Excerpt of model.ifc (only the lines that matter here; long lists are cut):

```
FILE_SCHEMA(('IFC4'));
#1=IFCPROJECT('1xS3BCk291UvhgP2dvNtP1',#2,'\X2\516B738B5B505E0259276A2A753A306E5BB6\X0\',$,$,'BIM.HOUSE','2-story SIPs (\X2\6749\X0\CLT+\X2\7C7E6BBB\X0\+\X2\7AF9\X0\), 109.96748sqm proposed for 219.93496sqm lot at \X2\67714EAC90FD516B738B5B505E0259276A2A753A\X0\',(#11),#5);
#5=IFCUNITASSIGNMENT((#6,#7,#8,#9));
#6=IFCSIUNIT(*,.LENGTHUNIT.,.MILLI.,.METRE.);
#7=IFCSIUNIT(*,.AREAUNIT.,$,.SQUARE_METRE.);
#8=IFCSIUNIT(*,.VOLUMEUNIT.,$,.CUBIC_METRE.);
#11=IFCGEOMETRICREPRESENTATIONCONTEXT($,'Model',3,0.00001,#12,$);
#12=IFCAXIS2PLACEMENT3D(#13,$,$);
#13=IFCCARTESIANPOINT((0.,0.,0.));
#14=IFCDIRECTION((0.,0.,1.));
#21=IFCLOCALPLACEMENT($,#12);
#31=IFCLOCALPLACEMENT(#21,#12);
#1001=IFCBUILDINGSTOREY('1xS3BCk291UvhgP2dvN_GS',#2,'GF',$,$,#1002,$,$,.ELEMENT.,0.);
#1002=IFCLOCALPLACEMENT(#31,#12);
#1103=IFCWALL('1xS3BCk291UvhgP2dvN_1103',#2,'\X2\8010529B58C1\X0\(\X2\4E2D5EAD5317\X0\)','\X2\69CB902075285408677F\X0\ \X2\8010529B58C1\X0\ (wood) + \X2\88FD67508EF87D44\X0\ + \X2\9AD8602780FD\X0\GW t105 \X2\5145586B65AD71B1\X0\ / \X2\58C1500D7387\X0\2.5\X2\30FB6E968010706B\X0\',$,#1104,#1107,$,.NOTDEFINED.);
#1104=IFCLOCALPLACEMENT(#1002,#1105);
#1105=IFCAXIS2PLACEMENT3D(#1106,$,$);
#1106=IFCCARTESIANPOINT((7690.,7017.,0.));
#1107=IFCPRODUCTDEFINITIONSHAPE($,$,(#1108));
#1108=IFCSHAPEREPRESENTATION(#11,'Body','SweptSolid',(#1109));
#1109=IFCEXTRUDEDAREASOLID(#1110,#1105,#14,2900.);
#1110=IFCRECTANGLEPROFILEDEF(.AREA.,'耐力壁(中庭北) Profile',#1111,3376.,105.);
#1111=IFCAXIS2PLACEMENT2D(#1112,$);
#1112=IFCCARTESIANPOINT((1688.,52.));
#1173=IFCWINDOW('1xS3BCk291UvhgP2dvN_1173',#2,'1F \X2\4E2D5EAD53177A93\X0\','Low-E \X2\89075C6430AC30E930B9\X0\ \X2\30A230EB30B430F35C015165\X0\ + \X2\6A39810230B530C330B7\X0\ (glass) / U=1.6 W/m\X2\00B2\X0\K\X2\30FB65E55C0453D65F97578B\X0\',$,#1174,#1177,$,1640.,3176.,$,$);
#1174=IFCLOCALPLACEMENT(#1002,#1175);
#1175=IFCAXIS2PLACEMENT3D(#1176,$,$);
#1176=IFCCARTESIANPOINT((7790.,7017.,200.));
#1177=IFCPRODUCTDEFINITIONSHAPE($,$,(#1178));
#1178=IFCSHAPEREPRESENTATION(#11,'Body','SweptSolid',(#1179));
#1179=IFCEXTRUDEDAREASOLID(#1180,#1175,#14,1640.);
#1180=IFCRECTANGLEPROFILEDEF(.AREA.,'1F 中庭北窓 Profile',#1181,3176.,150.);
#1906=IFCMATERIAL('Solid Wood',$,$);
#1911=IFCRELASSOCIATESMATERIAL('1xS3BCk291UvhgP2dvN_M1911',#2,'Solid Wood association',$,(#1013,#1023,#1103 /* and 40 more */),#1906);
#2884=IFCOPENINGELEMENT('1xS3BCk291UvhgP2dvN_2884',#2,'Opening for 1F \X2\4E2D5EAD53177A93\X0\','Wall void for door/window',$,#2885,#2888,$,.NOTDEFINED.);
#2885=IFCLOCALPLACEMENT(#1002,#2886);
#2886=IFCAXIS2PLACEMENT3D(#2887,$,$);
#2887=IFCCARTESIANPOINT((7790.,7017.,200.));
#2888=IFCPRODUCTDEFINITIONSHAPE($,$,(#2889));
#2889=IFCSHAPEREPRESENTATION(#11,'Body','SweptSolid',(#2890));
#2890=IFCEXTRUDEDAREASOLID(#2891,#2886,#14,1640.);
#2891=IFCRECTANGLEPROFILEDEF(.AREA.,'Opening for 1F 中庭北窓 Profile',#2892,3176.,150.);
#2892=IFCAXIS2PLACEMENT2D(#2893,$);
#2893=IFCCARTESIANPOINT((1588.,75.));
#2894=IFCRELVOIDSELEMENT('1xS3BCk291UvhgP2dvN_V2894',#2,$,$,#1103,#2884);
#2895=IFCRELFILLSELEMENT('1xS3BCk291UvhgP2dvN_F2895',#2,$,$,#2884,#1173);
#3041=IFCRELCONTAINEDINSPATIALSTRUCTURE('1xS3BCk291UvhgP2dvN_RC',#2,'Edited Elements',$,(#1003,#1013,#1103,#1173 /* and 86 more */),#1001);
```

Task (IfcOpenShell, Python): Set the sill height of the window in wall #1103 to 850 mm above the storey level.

```python
import numpy as np
import ifcopenshell
import ifcopenshell.api.geometry
import ifcopenshell.geom
import ifcopenshell.util.element
import ifcopenshell.util.placement
import ifcopenshell.util.shape
import ifcopenshell.util.unit

model = ifcopenshell.open("model.ifc")
unit_scale = ifcopenshell.util.unit.calculate_unit_scale(model)

window = model.by_id(1173)
opening = window.FillsVoids[0].RelatingOpeningElement
storey = ifcopenshell.util.element.get_container(window, ifc_class="IfcBuildingStorey")
level = ifcopenshell.util.placement.get_local_placement(storey.ObjectPlacement)[2, 3]

# The opening's origin need not be at the sill, so measure its lowest point.
shape = ifcopenshell.geom.create_shape(ifcopenshell.geom.settings(), opening)
bottom = ifcopenshell.util.shape.get_shape_bottom_elevation(shape, shape.geometry) / unit_scale
dz = level + 0.85 / unit_scale - bottom

shift = np.array([0.0, 0.0, dz])
# The window is not placed relative to its opening, so move both.
for product in (opening, window):
    matrix = ifcopenshell.util.placement.get_local_placement(product.ObjectPlacement)
    matrix[:3, 3] += shift
    ifcopenshell.api.geometry.edit_object_placement(model, product=product, matrix=matrix, is_si=False)

print(f"moved by {dz * unit_scale:+.3f} m")

model.write("model_edited.ifc")
```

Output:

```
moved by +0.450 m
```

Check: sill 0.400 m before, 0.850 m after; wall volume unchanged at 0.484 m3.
